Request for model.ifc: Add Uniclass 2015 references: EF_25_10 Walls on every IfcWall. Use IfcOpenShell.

First a look at what the model holds.

```python
import ifcopenshell

model = ifcopenshell.open("model.ifc")
print(model.schema)
print("classifications:", [c.Name for c in model.by_type("IfcClassification")])
for ifc_class in ("IfcDoor", "IfcRoof", "IfcStair", "IfcWall", "IfcWindow"):
    print(ifc_class, len(model.by_type(ifc_class)))
```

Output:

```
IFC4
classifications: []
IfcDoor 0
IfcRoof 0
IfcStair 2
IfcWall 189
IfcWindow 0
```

```python
import ifcopenshell
import ifcopenshell.api.classification

model = ifcopenshell.open("model.ifc")

system = ifcopenshell.api.classification.add_classification(model, classification="Uniclass 2015")

codes = {
    "IfcWall": ("EF_25_10", "Walls"),
}
for ifc_class, (code, name) in codes.items():
    products = model.by_type(ifc_class)
    ifcopenshell.api.classification.add_reference(
        model, products=products, classification=system, identification=code, name=name
    )
    print(code, len(products))

model.write("model_v2.ifc")
```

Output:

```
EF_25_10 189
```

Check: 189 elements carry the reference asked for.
